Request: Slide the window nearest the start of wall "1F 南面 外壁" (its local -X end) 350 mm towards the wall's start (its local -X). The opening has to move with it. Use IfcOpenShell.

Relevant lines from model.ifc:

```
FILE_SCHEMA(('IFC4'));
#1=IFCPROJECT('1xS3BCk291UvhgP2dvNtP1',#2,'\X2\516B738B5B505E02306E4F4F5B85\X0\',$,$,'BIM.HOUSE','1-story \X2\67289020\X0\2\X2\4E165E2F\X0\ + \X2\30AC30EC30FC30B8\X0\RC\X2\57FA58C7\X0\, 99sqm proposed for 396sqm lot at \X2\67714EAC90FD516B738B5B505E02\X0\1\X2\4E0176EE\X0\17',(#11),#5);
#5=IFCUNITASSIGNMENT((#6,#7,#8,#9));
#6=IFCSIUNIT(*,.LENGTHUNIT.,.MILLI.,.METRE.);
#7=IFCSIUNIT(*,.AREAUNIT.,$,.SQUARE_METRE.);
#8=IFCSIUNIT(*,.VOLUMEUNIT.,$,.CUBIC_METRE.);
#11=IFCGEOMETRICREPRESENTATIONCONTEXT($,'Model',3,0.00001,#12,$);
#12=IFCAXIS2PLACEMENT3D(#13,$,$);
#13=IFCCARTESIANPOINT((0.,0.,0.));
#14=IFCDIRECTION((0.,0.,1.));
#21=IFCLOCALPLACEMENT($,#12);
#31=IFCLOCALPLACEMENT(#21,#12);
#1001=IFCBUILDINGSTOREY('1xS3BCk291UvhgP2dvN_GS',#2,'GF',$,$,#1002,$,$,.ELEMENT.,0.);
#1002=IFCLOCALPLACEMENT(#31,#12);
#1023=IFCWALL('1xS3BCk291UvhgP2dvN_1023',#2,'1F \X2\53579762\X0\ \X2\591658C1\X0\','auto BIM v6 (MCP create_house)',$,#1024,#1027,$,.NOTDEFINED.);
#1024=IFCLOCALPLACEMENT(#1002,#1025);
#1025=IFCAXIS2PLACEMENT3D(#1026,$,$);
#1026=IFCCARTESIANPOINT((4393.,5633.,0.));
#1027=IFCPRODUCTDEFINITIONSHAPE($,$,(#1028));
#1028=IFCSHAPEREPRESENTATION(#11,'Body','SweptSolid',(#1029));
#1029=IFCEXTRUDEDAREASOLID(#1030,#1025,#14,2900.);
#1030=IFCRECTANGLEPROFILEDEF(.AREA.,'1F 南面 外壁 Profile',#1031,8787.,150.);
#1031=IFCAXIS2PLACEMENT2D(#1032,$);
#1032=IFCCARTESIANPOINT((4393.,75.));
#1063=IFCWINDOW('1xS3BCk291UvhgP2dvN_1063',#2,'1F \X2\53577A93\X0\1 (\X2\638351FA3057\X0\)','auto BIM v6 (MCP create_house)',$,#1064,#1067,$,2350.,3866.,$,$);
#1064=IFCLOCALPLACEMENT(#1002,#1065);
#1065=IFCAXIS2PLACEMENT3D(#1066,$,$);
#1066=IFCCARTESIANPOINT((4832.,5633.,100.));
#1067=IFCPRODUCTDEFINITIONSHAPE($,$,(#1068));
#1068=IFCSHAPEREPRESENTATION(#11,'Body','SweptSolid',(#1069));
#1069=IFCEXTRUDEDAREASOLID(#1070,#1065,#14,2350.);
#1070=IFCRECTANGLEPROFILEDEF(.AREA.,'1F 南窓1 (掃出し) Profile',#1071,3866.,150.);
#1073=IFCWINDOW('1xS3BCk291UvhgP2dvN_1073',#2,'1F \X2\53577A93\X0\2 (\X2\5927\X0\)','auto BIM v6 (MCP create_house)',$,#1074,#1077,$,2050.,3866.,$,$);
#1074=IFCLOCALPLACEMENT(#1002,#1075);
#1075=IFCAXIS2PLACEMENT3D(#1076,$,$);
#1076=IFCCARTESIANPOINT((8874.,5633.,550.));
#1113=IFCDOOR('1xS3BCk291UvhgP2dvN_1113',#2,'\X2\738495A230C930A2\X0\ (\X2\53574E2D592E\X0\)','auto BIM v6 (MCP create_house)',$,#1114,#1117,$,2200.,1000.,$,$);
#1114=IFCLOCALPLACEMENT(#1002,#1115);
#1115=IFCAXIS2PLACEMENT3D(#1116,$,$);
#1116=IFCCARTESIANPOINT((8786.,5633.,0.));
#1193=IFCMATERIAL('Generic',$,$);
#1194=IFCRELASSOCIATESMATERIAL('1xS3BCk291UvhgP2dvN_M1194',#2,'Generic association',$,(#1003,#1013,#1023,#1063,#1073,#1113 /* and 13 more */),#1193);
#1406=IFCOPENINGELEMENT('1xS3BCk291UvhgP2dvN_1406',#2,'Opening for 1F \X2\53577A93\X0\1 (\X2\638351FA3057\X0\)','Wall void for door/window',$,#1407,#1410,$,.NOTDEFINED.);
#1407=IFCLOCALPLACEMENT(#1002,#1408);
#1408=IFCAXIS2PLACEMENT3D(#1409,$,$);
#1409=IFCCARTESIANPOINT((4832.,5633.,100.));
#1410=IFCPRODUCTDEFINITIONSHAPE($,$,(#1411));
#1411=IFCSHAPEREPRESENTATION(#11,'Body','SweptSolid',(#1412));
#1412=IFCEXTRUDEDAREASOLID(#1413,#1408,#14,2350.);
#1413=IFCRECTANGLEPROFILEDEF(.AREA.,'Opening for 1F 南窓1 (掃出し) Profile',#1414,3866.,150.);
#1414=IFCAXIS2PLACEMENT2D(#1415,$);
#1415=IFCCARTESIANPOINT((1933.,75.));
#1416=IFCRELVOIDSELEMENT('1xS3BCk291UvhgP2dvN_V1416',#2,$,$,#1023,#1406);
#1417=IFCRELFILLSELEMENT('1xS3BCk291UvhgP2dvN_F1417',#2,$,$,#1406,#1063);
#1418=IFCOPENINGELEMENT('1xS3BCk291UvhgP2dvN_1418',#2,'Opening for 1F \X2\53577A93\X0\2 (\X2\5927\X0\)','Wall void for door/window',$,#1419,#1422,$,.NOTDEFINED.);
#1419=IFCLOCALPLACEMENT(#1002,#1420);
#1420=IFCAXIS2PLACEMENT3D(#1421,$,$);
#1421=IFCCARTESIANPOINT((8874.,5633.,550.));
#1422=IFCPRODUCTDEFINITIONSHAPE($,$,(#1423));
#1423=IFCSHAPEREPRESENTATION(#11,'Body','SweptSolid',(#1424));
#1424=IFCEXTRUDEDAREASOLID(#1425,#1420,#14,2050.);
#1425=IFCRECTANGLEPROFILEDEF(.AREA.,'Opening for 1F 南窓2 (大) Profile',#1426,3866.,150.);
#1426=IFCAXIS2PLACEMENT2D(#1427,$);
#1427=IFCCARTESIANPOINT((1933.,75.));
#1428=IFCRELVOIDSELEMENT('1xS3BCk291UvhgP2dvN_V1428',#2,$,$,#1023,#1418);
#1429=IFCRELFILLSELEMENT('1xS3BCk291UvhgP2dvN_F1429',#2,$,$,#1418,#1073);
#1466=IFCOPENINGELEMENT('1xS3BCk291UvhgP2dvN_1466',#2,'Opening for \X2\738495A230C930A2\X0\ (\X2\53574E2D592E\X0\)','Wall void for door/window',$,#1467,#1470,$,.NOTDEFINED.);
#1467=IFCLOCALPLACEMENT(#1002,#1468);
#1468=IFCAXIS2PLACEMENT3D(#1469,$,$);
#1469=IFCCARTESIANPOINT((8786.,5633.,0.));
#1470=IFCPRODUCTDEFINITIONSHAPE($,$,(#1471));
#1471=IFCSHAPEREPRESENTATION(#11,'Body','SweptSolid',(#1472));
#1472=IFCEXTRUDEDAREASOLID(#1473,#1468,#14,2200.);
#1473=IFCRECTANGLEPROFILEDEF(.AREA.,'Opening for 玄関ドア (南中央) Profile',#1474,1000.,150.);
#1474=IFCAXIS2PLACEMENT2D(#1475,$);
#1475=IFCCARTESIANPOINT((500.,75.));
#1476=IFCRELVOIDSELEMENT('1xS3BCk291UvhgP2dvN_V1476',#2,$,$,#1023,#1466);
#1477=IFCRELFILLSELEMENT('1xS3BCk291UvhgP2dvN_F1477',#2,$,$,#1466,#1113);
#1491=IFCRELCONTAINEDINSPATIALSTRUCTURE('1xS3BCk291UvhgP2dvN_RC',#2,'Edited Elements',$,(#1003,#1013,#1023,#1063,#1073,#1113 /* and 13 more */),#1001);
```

```python
import ifcopenshell
import ifcopenshell.api.geometry
import ifcopenshell.util.placement
import ifcopenshell.util.unit

model = ifcopenshell.open("model.ifc")
unit_scale = ifcopenshell.util.unit.calculate_unit_scale(model)

window = model.by_guid("1xS3BCk291UvhgP2dvN_1063")
opening = window.FillsVoids[0].RelatingOpeningElement
wall = opening.VoidsElements[0].RelatingBuildingElement

wall_matrix = ifcopenshell.util.placement.get_local_placement(wall.ObjectPlacement)
shift = wall_matrix[:3, 0] * -0.35 / unit_scale
before = ifcopenshell.util.placement.get_local_placement(window.ObjectPlacement)[:3, 3].copy()

# The window is not placed relative to its opening, so move both.
for product in (opening, window):
    matrix = ifcopenshell.util.placement.get_local_placement(product.ObjectPlacement)
    matrix[:3, 3] += shift
    ifcopenshell.api.geometry.edit_object_placement(model, product=product, matrix=matrix, is_si=False)

after = ifcopenshell.util.placement.get_local_placement(window.ObjectPlacement)[:3, 3]
print("window moved by", (after - before).round(3) + 0.0)

model.write("model_v2.ifc")
```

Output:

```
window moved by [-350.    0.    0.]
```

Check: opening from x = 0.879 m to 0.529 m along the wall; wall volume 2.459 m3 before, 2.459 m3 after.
